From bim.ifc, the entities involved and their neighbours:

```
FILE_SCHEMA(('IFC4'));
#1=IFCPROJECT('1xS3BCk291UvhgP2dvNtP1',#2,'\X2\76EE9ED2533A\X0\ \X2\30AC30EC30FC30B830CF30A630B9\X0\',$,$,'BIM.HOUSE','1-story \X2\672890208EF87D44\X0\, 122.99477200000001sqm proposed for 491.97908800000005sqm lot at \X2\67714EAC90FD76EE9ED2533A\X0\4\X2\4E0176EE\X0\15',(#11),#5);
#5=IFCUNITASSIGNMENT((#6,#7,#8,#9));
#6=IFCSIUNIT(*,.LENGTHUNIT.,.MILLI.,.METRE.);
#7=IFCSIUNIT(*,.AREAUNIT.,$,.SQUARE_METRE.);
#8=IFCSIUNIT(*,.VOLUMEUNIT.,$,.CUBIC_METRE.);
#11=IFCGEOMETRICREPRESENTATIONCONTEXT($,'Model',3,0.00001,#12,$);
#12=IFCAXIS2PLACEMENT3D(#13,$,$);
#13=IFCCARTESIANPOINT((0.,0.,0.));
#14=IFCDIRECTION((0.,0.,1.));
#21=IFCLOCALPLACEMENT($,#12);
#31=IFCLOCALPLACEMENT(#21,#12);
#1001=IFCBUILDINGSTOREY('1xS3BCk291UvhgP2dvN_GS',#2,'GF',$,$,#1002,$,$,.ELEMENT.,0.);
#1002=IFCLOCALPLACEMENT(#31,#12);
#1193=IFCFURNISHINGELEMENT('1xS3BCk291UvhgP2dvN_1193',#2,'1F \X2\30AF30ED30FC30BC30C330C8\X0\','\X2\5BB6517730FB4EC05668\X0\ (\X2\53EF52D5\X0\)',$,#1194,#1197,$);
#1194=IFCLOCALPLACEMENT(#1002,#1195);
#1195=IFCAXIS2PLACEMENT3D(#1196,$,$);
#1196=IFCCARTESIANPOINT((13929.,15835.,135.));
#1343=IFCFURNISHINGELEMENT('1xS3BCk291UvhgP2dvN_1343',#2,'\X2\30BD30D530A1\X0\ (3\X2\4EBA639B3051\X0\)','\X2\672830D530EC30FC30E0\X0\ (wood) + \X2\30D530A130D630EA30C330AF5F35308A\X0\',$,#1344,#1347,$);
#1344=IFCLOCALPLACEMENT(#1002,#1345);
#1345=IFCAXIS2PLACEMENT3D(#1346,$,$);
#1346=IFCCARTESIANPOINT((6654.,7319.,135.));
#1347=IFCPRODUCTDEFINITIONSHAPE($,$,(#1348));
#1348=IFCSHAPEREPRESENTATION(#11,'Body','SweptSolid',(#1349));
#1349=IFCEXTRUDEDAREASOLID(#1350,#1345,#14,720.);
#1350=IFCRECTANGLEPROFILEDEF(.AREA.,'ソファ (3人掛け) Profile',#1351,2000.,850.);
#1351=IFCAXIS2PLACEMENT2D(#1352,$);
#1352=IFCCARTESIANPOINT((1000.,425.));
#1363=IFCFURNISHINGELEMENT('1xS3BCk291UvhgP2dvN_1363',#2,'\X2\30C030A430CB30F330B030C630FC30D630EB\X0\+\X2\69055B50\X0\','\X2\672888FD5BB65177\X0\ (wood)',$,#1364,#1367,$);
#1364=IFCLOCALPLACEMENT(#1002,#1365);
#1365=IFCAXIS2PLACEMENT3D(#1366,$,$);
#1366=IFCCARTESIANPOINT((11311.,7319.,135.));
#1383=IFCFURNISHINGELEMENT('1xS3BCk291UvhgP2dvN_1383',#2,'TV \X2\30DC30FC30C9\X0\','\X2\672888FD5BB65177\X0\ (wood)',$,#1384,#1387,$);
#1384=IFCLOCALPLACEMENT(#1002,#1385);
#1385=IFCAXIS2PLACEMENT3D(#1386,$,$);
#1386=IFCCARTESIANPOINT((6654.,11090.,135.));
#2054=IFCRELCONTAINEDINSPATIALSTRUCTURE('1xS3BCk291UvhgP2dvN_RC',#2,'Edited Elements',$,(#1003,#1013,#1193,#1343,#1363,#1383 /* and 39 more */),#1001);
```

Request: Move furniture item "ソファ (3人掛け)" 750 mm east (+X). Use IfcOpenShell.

```python
import ifcopenshell
import ifcopenshell.api.geometry
import ifcopenshell.util.placement
import ifcopenshell.util.unit

model = ifcopenshell.open("bim.ifc")
unit_scale = ifcopenshell.util.unit.calculate_unit_scale(model)

item = model.by_guid("1xS3BCk291UvhgP2dvN_1343")
matrix = ifcopenshell.util.placement.get_local_placement(item.ObjectPlacement)
matrix[0, 3] += 0.75 / unit_scale
ifcopenshell.api.geometry.edit_object_placement(model, product=item, matrix=matrix, is_si=False)

print(ifcopenshell.util.placement.get_local_placement(item.ObjectPlacement).round(3) + 0.0)

model.write("bim_rev.ifc")
```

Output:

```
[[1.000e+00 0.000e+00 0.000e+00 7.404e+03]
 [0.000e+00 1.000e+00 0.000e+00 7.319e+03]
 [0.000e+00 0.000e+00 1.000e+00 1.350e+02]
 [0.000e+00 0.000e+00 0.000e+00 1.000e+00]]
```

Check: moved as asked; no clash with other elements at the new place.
